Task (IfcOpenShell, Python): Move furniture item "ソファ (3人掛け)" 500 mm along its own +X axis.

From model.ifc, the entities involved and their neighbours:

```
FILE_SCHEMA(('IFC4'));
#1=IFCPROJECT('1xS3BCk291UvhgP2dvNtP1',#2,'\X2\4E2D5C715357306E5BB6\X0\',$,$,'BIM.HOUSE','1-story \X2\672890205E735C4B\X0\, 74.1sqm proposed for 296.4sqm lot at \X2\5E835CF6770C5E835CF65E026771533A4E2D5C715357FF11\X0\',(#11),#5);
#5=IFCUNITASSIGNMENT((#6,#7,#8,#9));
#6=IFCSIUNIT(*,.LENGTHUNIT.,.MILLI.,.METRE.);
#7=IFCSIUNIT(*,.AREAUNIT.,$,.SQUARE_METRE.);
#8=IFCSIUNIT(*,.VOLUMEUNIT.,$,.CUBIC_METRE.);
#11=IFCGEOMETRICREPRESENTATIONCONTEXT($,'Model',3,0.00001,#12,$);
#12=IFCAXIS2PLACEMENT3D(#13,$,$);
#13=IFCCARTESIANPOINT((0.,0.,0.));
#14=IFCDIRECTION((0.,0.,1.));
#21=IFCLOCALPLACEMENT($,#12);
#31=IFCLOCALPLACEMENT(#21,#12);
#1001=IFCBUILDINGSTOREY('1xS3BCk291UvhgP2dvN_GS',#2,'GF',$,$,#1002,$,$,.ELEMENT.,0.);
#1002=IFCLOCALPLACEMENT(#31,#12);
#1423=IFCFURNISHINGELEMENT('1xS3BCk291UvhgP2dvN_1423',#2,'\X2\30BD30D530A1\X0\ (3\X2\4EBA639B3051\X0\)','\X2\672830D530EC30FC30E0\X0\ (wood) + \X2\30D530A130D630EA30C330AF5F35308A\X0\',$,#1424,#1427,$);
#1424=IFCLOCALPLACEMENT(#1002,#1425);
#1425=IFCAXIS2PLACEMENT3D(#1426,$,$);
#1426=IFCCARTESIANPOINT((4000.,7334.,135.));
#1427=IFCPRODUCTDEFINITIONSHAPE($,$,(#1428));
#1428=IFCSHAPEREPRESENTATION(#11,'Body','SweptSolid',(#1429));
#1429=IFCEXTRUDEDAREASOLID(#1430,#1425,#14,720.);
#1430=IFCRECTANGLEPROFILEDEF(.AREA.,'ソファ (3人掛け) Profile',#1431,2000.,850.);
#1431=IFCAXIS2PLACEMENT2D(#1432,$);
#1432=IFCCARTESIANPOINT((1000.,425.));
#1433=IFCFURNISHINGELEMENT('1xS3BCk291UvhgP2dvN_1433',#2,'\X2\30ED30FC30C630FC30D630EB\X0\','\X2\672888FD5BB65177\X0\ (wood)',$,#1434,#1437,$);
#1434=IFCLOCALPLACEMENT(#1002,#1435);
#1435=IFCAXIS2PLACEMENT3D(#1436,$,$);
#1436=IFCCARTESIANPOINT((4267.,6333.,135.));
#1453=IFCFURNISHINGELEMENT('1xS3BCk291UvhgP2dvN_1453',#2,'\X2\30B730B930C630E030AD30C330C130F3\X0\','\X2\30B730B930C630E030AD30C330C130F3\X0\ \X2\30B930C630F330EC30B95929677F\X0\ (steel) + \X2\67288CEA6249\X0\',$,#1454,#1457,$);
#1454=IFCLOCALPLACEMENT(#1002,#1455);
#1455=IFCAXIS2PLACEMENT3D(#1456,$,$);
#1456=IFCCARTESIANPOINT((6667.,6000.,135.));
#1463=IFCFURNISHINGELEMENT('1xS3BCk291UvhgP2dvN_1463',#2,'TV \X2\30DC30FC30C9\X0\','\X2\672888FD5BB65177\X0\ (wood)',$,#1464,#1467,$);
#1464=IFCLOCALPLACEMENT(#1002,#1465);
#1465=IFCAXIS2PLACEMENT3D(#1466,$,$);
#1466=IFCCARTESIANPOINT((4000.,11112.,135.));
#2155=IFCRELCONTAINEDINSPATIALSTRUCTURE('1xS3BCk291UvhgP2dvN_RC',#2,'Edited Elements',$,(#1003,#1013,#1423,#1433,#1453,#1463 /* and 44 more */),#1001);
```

```python
import ifcopenshell
import ifcopenshell.api.geometry
import ifcopenshell.util.placement
import ifcopenshell.util.unit

model = ifcopenshell.open("model.ifc")
unit_scale = ifcopenshell.util.unit.calculate_unit_scale(model)

item = model.by_id(1423)
matrix = ifcopenshell.util.placement.get_local_placement(item.ObjectPlacement)
matrix[:3, 3] += matrix[:3, 0] * 0.5 / unit_scale
ifcopenshell.api.geometry.edit_object_placement(model, product=item, matrix=matrix, is_si=False)

print(ifcopenshell.util.placement.get_local_placement(item.ObjectPlacement).round(3) + 0.0)

model.write("model_v2.ifc")
```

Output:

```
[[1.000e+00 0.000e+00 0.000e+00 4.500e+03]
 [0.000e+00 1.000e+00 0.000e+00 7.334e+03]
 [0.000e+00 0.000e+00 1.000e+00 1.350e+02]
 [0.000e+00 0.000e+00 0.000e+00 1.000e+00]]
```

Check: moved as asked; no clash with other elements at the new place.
